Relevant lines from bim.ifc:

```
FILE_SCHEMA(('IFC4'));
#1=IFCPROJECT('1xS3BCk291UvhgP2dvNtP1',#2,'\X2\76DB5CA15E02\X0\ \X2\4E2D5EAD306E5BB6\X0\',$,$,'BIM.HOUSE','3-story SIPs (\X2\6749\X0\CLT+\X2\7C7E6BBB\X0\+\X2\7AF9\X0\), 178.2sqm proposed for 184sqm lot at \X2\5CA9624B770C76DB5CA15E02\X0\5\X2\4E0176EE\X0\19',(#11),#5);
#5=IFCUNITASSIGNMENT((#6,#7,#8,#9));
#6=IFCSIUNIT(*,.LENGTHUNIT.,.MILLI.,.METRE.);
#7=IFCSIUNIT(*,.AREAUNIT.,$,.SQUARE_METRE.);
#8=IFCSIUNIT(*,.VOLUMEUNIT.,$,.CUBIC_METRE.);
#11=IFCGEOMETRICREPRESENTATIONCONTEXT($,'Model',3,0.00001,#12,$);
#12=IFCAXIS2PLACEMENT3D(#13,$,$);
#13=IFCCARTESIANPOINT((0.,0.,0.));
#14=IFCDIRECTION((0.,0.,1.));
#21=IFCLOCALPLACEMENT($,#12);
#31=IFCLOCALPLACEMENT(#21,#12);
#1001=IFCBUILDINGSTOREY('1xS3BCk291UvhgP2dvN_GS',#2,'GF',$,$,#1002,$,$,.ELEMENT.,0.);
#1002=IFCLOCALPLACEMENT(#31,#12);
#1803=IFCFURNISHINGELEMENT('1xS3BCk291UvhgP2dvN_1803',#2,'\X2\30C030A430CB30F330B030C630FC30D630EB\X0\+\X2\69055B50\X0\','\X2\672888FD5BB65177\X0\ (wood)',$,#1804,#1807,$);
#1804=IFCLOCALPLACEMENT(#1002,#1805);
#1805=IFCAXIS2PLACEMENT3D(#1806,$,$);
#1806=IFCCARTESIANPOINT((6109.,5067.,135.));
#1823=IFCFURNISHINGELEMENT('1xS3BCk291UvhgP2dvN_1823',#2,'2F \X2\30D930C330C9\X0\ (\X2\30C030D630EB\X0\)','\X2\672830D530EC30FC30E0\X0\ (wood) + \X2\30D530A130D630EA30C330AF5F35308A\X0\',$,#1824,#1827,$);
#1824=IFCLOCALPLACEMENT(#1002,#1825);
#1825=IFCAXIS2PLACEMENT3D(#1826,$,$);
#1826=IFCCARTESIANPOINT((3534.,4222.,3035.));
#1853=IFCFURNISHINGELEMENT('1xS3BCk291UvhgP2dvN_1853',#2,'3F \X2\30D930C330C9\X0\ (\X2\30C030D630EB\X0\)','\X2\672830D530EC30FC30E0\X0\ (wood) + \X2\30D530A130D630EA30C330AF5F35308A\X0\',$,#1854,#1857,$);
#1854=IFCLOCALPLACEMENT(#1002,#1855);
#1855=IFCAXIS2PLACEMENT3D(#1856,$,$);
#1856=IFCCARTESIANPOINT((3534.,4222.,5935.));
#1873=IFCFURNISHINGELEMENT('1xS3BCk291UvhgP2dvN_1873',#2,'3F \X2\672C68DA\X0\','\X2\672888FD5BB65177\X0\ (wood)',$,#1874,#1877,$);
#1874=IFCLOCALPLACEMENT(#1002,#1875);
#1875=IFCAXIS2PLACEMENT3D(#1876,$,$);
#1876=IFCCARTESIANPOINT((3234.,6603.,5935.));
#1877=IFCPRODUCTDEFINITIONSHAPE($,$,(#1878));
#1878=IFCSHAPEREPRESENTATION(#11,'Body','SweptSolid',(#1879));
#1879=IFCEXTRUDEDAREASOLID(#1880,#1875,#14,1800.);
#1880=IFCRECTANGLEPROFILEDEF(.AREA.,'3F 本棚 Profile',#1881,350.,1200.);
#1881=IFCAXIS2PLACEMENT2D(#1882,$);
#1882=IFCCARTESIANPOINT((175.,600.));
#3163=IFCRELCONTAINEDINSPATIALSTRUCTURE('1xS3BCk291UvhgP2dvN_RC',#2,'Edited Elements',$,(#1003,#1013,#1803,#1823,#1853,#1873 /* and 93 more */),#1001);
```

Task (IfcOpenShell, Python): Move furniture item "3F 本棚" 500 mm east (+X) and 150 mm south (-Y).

```python
import ifcopenshell
import ifcopenshell.api.geometry
import ifcopenshell.util.placement

model = ifcopenshell.open("bim.ifc")

item = model.by_guid("1xS3BCk291UvhgP2dvN_1873")
matrix = ifcopenshell.util.placement.get_local_placement(item.ObjectPlacement)
matrix[0, 3] += 500.0
matrix[1, 3] -= 150.0
ifcopenshell.api.geometry.edit_object_placement(model, product=item, matrix=matrix, is_si=False)

print(ifcopenshell.util.placement.get_local_placement(item.ObjectPlacement).round(3) + 0.0)

model.write("bim_edited.ifc")
```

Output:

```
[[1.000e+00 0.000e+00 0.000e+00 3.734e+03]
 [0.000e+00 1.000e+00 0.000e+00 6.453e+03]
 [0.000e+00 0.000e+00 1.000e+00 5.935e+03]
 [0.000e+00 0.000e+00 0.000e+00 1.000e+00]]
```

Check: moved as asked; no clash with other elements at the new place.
